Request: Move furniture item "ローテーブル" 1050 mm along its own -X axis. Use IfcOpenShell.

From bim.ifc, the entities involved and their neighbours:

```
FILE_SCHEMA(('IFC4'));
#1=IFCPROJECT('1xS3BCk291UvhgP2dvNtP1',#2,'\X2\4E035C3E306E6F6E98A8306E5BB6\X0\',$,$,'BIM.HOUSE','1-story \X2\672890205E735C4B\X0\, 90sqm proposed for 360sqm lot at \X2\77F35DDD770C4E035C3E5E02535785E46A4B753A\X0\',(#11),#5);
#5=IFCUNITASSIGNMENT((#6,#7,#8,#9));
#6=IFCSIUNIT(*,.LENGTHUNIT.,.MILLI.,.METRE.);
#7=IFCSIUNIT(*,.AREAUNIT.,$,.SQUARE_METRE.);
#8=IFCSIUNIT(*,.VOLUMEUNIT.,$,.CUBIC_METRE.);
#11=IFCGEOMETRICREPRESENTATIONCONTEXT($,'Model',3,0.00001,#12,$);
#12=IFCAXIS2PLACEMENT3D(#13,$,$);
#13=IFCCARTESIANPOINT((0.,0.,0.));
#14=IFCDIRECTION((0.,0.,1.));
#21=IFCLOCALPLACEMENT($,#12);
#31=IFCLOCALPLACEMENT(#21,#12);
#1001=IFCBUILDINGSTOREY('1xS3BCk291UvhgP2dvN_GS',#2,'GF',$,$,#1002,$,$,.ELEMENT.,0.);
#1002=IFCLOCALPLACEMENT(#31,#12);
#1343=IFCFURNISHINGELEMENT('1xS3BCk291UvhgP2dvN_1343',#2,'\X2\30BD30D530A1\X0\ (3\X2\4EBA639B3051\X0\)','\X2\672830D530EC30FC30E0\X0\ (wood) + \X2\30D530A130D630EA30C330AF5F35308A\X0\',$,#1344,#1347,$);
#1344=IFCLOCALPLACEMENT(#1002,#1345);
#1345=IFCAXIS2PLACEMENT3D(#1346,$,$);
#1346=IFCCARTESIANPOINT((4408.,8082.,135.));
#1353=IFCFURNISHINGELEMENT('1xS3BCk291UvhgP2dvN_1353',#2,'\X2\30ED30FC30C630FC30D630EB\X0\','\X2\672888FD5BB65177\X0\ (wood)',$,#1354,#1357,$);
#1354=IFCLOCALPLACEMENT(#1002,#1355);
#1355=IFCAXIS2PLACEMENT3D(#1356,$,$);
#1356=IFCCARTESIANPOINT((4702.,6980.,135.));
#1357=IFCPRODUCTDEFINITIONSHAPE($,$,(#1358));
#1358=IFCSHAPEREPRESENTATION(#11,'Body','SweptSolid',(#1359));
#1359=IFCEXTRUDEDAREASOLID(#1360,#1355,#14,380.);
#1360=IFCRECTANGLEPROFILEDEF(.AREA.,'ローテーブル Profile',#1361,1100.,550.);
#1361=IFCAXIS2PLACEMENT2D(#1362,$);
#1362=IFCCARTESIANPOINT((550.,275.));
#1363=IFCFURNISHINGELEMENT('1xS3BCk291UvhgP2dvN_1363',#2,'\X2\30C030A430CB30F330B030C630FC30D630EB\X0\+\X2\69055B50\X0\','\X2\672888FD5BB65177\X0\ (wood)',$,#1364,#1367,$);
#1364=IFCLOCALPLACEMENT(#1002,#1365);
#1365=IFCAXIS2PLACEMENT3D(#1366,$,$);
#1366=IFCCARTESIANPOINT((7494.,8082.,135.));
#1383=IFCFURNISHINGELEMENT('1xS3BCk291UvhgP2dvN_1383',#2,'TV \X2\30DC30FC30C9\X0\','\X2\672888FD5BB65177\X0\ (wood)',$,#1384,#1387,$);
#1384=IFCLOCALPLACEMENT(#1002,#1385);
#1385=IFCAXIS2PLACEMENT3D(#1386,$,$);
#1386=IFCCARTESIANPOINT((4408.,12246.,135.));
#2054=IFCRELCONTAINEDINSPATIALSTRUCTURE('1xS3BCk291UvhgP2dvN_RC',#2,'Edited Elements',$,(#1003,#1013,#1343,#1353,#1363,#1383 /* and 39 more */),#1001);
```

```python
import ifcopenshell
import ifcopenshell.api.geometry
import ifcopenshell.util.placement
import ifcopenshell.util.unit

model = ifcopenshell.open("bim.ifc")
unit_scale = ifcopenshell.util.unit.calculate_unit_scale(model)

item = model.by_id(1353)
matrix = ifcopenshell.util.placement.get_local_placement(item.ObjectPlacement)
matrix[:3, 3] -= matrix[:3, 0] * 1.05 / unit_scale
ifcopenshell.api.geometry.edit_object_placement(model, product=item, matrix=matrix, is_si=False)

print(ifcopenshell.util.placement.get_local_placement(item.ObjectPlacement).round(3) + 0.0)

model.write("bim_edited.ifc")
```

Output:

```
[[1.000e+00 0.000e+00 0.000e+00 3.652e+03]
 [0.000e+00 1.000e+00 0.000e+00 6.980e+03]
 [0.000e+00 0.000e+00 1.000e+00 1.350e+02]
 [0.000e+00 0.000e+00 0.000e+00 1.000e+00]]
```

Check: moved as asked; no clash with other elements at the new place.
